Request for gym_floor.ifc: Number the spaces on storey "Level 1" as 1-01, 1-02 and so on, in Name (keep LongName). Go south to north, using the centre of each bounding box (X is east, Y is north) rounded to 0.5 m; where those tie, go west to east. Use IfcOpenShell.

First a look at what the model holds.

```python
import ifcopenshell
import ifcopenshell.util.element
import ifcopenshell.util.placement

model = ifcopenshell.open("gym_floor.ifc")
print(model.schema)
storey = next(s for s in model.by_type("IfcBuildingStorey") if s.Name == "Level 1")
spaces = [e for e in ifcopenshell.util.element.get_decomposition(storey) if e.is_a("IfcSpace")]
for e in sorted(spaces, key=lambda e: e.id()):
    origin = ifcopenshell.util.placement.get_local_placement(e.ObjectPlacement)[:3, 3]
    print(e.id(), e.Name, e.LongName, origin.round(2) + 0.0, sep=" | ")
```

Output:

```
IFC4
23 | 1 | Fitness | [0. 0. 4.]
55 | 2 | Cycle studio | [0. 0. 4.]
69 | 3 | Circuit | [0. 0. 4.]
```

```python
import ifcopenshell
import ifcopenshell.geom
import ifcopenshell.util.element
import ifcopenshell.util.shape

model = ifcopenshell.open("gym_floor.ifc")
settings = ifcopenshell.geom.settings()
settings.set("use-world-coords", True)


def centre(element):
    shape = ifcopenshell.geom.create_shape(settings, element)
    return ifcopenshell.util.shape.get_bbox_centroid(shape.geometry)


storey = next(s for s in model.by_type("IfcBuildingStorey") if s.Name == "Level 1")
spaces = [e for e in ifcopenshell.util.element.get_decomposition(storey) if e.is_a("IfcSpace")]

# Insertion points can sit at a corner or the storey origin, so sort by the geometry (in metres).
centres = {e: centre(e) for e in spaces}
spaces.sort(key=lambda e: (round(centres[e][1] / 0.5), centres[e][0]))

for i, e in enumerate(spaces, start=1):
    number = f"1-{i:02d}"
    e.Name = number
    print(e.id(), number)

model.write("gym_floor-out.ifc")
```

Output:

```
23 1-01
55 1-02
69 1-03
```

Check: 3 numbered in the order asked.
